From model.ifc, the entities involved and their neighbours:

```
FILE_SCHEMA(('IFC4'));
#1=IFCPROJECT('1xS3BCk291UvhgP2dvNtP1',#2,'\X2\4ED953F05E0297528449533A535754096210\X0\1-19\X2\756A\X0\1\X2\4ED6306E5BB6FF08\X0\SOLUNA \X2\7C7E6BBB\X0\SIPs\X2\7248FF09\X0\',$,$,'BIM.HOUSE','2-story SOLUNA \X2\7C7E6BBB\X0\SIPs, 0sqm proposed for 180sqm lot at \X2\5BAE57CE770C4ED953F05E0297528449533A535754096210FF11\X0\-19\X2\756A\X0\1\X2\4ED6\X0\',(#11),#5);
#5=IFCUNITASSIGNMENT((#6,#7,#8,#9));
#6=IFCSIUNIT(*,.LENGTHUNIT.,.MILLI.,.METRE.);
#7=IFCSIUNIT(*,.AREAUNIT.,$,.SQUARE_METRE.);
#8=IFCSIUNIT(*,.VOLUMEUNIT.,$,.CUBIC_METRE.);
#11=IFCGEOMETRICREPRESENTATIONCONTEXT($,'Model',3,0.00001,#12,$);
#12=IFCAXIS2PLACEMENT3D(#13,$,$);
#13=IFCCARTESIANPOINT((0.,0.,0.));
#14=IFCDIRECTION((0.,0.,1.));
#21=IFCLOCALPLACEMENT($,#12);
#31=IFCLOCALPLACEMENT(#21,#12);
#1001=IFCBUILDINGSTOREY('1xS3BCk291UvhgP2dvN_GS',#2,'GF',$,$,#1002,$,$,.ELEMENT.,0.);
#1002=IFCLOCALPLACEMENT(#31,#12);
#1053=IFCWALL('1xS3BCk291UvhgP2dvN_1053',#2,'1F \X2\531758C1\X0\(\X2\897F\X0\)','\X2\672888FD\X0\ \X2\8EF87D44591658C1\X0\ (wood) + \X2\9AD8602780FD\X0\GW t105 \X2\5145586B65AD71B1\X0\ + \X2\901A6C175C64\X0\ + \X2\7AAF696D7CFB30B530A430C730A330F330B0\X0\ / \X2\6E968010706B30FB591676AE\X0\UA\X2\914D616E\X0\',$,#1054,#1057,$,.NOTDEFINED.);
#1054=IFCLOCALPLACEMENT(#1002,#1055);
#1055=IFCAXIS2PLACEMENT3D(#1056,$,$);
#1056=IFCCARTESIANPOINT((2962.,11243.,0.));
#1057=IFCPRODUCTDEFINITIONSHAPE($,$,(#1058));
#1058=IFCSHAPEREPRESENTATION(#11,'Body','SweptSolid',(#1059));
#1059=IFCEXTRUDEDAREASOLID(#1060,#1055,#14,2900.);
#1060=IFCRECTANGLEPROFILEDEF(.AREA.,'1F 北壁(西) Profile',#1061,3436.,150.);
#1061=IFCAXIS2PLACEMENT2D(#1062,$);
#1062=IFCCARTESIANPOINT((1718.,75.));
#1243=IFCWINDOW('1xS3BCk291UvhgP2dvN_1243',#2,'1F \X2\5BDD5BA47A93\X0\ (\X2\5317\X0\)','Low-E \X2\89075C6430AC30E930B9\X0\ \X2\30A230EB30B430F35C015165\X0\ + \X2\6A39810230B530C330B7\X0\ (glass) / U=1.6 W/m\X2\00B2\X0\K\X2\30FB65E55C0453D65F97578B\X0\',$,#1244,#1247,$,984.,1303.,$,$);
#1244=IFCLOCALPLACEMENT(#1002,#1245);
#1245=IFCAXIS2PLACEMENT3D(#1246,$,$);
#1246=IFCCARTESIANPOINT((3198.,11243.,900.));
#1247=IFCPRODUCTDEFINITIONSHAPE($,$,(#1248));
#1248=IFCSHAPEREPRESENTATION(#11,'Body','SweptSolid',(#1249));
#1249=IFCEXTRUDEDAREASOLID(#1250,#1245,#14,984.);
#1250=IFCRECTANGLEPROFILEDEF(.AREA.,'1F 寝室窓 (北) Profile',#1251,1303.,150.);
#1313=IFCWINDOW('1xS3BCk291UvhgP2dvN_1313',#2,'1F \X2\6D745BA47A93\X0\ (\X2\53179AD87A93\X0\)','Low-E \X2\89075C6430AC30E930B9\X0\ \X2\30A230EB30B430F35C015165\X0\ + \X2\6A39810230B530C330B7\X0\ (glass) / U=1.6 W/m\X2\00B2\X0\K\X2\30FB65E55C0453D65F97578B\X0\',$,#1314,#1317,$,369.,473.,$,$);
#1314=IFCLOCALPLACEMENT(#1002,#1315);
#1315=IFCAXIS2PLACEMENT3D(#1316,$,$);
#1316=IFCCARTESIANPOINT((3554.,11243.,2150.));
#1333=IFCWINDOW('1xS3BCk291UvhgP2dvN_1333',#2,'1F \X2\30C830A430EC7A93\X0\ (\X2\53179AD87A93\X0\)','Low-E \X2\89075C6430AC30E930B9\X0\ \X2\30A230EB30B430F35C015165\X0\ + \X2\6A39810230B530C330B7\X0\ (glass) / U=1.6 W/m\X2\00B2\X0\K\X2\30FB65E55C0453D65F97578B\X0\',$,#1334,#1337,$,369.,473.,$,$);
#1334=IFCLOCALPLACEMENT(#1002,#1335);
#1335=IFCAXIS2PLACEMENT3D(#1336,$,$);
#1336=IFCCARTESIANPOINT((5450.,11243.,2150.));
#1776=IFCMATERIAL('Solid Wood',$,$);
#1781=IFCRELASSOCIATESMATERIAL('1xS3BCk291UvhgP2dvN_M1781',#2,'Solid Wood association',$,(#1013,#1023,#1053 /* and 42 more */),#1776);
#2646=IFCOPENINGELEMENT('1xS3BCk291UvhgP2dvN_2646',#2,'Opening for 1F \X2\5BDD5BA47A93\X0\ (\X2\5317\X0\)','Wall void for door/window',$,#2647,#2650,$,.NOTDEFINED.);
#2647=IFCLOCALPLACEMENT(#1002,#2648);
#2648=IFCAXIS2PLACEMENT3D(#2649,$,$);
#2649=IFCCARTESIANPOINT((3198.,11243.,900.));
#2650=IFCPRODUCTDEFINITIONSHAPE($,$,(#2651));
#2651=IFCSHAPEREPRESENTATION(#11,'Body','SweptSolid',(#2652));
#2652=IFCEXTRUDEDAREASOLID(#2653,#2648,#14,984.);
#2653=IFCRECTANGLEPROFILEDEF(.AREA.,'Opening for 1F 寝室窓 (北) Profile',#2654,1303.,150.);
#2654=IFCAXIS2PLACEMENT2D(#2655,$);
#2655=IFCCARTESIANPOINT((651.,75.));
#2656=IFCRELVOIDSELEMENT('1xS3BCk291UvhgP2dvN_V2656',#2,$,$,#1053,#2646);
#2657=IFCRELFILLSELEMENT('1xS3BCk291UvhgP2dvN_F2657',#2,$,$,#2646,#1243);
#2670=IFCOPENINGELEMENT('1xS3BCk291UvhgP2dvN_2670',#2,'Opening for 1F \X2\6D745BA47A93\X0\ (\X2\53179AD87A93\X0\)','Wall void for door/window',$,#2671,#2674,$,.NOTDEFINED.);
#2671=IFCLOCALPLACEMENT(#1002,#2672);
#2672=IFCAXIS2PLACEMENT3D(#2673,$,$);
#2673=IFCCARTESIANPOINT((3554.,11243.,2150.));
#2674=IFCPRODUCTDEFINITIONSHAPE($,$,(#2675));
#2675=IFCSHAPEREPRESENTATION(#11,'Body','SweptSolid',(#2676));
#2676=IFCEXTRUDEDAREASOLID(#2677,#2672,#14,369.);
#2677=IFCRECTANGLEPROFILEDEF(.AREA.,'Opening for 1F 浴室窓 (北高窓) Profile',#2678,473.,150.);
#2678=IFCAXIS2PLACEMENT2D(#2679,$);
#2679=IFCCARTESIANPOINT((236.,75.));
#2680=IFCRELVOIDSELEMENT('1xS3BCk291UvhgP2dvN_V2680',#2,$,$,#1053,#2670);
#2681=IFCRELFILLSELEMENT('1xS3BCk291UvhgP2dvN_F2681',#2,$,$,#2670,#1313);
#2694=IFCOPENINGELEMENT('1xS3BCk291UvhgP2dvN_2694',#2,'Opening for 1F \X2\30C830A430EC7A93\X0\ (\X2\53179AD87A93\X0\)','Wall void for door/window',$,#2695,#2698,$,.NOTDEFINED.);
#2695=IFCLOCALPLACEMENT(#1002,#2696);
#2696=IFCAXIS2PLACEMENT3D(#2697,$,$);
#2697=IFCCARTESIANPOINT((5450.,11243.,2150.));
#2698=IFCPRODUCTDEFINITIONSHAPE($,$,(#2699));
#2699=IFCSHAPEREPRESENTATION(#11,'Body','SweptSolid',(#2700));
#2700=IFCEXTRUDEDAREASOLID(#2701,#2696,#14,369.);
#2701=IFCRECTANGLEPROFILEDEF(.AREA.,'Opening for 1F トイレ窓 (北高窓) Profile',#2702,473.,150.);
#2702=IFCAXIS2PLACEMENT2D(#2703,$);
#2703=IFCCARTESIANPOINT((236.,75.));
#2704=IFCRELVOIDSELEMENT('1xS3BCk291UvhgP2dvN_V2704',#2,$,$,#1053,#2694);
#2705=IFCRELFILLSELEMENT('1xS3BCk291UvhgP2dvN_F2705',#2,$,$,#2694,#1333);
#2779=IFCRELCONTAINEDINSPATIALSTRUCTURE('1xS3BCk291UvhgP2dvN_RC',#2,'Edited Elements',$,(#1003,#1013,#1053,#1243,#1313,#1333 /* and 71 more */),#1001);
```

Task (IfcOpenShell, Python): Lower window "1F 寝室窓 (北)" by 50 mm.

```python
import numpy as np
import ifcopenshell
import ifcopenshell.api.geometry
import ifcopenshell.util.placement
import ifcopenshell.util.unit

model = ifcopenshell.open("model.ifc")
unit_scale = ifcopenshell.util.unit.calculate_unit_scale(model)

window = model.by_id(1243)
opening = window.FillsVoids[0].RelatingOpeningElement
dz = -50.0

shift = np.array([0.0, 0.0, dz])
# The window is not placed relative to its opening, so move both.
for product in (opening, window):
    matrix = ifcopenshell.util.placement.get_local_placement(product.ObjectPlacement)
    matrix[:3, 3] += shift
    ifcopenshell.api.geometry.edit_object_placement(model, product=product, matrix=matrix, is_si=False)

print(f"moved by {dz * unit_scale:+.3f} m")

model.write("model_updated.ifc")
```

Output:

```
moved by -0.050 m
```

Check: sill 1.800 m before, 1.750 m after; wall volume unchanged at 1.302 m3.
